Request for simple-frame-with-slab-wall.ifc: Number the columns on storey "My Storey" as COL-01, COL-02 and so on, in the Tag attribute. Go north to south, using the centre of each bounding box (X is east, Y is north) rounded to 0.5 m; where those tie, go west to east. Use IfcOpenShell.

First a look at what the model holds.

```python
import ifcopenshell
import ifcopenshell.util.element
import ifcopenshell.util.placement

model = ifcopenshell.open("simple-frame-with-slab-wall.ifc")
print(model.schema)
storey = next(s for s in model.by_type("IfcBuildingStorey") if s.Name == "My Storey")
columns = [e for e in ifcopenshell.util.element.get_decomposition(storey) if e.is_a("IfcColumn")]
for e in sorted(columns, key=lambda e: e.id()):
    origin = ifcopenshell.util.placement.get_local_placement(e.ObjectPlacement)[:3, 3]
    print(e.id(), e.Tag, e.Name, origin.round(2) + 0.0, sep=" | ")
```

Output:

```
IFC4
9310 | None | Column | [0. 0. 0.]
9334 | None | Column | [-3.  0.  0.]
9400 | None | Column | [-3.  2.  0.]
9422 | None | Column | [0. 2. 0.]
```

```python
import ifcopenshell
import ifcopenshell.geom
import ifcopenshell.util.element
import ifcopenshell.util.shape

model = ifcopenshell.open("simple-frame-with-slab-wall.ifc")
settings = ifcopenshell.geom.settings()
settings.set("use-world-coords", True)


def centre(element):
    shape = ifcopenshell.geom.create_shape(settings, element)
    return ifcopenshell.util.shape.get_bbox_centroid(shape.geometry)


storey = next(s for s in model.by_type("IfcBuildingStorey") if s.Name == "My Storey")
columns = [e for e in ifcopenshell.util.element.get_decomposition(storey) if e.is_a("IfcColumn")]

# Insertion points can sit at a corner or the storey origin, so sort by the geometry (in metres).
centres = {e: centre(e) for e in columns}
columns.sort(key=lambda e: (-round(centres[e][1] / 0.5), centres[e][0]))

for i, e in enumerate(columns, start=1):
    number = f"COL-{i:02d}"
    e.Tag = number
    print(e.id(), number)

model.write("simple-frame-with-slab-wall-out.ifc")
```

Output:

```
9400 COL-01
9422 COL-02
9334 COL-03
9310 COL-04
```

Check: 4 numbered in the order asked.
